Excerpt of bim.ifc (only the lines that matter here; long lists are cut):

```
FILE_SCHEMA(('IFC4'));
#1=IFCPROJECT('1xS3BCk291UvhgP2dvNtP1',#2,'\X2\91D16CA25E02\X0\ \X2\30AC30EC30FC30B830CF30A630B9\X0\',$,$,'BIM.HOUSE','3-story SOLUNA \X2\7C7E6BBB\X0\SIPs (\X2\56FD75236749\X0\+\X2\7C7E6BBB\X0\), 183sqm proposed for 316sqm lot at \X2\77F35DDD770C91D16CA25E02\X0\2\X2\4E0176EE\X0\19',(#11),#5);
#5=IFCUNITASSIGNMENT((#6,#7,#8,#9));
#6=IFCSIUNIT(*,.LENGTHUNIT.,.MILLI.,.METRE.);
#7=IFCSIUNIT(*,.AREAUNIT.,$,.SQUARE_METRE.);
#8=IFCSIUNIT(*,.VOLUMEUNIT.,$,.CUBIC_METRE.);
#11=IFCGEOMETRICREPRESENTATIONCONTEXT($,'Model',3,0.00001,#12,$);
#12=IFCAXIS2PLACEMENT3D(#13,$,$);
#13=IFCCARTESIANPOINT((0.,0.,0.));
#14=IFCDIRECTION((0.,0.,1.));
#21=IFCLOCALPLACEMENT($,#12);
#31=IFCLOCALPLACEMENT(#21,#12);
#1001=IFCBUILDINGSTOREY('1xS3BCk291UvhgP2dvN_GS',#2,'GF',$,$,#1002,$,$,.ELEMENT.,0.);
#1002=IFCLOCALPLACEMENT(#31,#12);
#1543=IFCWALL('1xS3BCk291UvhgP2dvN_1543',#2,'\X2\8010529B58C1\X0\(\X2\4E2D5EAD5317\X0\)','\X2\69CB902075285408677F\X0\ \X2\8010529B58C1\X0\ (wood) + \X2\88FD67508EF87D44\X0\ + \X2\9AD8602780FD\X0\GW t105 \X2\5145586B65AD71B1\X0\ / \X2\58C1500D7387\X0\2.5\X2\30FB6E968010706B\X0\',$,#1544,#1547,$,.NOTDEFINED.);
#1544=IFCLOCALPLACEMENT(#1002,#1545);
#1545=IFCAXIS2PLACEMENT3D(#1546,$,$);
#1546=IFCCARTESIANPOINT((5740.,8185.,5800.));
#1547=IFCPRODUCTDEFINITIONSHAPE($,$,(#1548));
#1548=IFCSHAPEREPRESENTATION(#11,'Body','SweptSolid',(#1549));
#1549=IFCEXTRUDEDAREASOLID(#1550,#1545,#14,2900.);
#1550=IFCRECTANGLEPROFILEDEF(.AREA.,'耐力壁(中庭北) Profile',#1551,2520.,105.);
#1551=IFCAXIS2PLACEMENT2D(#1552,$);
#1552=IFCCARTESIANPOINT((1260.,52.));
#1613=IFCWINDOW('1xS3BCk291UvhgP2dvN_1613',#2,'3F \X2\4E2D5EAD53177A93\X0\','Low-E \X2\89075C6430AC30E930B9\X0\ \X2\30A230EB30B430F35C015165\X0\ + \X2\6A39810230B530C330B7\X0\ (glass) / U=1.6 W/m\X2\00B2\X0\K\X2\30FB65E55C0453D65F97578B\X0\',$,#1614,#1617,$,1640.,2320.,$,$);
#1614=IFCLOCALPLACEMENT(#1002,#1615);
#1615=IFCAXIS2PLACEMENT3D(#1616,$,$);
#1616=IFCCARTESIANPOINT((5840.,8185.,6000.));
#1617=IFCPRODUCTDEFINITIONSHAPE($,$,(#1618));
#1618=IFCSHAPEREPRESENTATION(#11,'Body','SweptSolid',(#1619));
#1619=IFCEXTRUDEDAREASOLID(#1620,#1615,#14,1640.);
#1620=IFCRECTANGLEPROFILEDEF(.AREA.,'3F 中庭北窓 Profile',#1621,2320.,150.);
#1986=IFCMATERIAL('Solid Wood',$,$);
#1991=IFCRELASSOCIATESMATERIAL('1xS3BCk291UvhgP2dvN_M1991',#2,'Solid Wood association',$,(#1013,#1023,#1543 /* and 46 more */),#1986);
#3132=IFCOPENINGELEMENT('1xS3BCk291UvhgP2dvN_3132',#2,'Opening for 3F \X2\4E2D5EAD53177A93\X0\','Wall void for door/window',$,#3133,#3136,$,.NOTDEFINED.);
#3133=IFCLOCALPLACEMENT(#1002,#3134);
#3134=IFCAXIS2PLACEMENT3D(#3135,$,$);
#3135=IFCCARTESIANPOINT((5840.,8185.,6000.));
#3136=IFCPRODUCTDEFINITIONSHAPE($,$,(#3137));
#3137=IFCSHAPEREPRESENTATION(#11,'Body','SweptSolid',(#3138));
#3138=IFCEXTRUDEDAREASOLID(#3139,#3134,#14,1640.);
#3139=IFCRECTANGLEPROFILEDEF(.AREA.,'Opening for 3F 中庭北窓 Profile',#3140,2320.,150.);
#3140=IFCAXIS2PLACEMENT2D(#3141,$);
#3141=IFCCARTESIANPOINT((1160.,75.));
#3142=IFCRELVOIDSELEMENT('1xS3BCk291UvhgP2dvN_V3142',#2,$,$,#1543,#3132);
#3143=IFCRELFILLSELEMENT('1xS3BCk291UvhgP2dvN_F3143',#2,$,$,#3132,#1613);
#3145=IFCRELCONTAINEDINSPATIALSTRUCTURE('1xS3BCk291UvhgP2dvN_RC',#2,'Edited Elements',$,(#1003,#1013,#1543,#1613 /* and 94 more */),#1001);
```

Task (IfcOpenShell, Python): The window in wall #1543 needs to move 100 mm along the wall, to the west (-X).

```python
import ifcopenshell
import ifcopenshell.api.geometry
import ifcopenshell.util.placement

model = ifcopenshell.open("bim.ifc")

window = model.by_guid("1xS3BCk291UvhgP2dvN_1613")
opening = window.FillsVoids[0].RelatingOpeningElement
wall = opening.VoidsElements[0].RelatingBuildingElement

wall_matrix = ifcopenshell.util.placement.get_local_placement(wall.ObjectPlacement)
shift = wall_matrix[:3, 0] * -100.0
before = ifcopenshell.util.placement.get_local_placement(window.ObjectPlacement)[:3, 3].copy()

# The window is not placed relative to its opening, so move both.
for product in (opening, window):
    matrix = ifcopenshell.util.placement.get_local_placement(product.ObjectPlacement)
    matrix[:3, 3] += shift
    ifcopenshell.api.geometry.edit_object_placement(model, product=product, matrix=matrix, is_si=False)

after = ifcopenshell.util.placement.get_local_placement(window.ObjectPlacement)[:3, 3]
print("window moved by", (after - before).round(3) + 0.0)

model.write("bim_rev.ifc")
```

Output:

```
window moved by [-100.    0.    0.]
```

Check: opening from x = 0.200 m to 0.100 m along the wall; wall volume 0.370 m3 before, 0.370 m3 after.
